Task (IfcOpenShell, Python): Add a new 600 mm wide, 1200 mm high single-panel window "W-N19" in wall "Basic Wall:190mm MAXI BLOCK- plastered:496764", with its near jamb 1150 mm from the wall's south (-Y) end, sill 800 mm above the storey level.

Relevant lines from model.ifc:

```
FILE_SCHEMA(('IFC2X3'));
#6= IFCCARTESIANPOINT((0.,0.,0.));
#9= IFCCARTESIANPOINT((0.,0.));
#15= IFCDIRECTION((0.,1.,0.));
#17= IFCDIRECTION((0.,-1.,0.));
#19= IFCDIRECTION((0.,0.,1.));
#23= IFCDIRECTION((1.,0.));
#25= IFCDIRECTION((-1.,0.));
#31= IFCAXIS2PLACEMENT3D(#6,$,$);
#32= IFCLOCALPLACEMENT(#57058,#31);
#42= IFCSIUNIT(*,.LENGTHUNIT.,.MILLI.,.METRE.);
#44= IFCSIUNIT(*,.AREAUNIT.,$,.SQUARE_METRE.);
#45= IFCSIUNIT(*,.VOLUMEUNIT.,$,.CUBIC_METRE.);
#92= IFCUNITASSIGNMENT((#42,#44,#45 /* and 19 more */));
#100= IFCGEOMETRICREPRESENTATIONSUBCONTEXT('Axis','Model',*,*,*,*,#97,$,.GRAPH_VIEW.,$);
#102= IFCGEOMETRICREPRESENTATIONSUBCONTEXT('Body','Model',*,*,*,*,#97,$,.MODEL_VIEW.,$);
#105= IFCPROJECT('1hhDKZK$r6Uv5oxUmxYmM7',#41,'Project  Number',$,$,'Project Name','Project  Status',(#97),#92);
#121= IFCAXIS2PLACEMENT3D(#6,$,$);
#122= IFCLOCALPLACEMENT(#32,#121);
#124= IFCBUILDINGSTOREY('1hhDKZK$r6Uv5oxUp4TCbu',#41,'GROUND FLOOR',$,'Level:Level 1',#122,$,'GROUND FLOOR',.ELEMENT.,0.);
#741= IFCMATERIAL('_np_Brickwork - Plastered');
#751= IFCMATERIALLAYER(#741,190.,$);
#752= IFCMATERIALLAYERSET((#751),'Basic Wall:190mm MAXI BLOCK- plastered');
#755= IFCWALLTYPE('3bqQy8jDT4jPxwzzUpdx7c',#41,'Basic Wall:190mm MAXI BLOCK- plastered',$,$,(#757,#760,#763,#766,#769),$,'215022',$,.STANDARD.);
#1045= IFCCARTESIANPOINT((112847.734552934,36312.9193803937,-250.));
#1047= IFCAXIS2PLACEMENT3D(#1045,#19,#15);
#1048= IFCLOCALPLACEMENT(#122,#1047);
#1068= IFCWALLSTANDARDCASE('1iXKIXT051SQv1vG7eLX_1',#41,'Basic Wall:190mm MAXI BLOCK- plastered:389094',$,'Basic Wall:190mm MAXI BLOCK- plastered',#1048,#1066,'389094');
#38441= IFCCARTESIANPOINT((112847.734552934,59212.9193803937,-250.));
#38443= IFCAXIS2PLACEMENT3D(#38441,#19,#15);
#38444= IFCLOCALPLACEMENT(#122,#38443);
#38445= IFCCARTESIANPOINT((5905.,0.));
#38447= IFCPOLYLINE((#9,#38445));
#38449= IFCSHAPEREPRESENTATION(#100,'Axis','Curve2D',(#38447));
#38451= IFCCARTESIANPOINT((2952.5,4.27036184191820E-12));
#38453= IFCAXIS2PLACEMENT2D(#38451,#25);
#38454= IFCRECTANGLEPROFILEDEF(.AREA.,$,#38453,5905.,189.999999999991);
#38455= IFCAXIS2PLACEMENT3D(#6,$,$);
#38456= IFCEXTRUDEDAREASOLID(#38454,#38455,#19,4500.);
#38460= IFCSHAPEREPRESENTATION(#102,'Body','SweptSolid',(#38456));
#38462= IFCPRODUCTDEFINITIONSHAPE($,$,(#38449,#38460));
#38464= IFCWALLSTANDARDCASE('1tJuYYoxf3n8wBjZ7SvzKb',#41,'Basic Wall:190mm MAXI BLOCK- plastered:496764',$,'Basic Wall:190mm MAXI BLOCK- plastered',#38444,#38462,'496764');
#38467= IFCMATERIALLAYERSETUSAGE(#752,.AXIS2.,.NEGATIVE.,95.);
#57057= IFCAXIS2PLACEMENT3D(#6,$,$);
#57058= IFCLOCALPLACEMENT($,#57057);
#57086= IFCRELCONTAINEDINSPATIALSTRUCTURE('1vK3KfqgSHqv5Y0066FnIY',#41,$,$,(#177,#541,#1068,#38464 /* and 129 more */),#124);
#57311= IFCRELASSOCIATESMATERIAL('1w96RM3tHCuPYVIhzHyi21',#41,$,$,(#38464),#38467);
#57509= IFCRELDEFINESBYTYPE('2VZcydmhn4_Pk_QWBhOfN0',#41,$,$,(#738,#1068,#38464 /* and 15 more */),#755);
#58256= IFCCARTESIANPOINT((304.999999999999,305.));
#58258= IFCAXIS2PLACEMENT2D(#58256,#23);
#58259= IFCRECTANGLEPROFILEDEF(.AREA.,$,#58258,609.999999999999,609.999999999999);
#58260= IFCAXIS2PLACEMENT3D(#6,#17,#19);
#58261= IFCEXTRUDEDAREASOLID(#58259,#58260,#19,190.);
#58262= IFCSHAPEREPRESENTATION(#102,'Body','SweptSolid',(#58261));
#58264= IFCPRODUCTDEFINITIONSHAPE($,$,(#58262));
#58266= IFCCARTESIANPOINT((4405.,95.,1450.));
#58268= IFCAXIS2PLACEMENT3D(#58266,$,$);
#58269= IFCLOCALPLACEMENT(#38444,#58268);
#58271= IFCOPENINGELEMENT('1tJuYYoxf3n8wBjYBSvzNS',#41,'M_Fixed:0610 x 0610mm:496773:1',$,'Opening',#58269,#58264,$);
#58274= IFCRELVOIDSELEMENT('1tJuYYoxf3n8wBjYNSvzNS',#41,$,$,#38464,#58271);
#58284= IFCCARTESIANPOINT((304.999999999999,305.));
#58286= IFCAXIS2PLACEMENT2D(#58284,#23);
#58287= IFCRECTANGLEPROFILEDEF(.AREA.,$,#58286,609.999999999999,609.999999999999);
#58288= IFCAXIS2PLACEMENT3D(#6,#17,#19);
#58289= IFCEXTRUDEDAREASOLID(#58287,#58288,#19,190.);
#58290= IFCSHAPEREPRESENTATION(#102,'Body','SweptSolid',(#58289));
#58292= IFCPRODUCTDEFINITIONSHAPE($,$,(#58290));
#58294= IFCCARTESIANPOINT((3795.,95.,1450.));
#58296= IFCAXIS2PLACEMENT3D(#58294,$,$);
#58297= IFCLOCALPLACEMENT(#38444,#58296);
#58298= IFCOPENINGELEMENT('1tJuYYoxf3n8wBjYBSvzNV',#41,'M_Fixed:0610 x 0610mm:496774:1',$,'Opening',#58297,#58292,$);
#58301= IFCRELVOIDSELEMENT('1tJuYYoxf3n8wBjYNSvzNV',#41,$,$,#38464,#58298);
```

```python
import numpy as np
import ifcopenshell
import ifcopenshell.api.feature
import ifcopenshell.api.geometry
import ifcopenshell.api.root
import ifcopenshell.api.spatial
import ifcopenshell.api.type
import ifcopenshell.geom
import ifcopenshell.util.element
import ifcopenshell.util.placement
import ifcopenshell.util.representation
import ifcopenshell.util.shape
import ifcopenshell.util.unit

model = ifcopenshell.open("model.ifc")
unit_scale = ifcopenshell.util.unit.calculate_unit_scale(model)
settings = ifcopenshell.geom.settings()


def volume(element):
    """Net volume in cubic metres, openings subtracted."""
    shape = ifcopenshell.geom.create_shape(settings, element)
    return ifcopenshell.util.shape.get_volume(shape.geometry)


wall = model.by_guid("1tJuYYoxf3n8wBjZ7SvzKb")
storey = ifcopenshell.util.element.get_container(wall, ifc_class="IfcBuildingStorey")
context = ifcopenshell.util.representation.get_context(model, "Model", "Body", "MODEL_VIEW")
before = volume(wall)

width, height, from_end, sill = 0.6, 1.2, 1.15, 0.8  # metres

# The wall runs along its own X axis, and the end named is its -X end.
wall_shape = ifcopenshell.geom.create_shape(settings, wall)
x, y, z = ifcopenshell.util.shape.get_vertices(wall_shape.geometry).T
start = x.min() + from_end
face, thickness = float(y.min()), float(y.max() - y.min())
wall_matrix = ifcopenshell.util.placement.get_local_placement(wall.ObjectPlacement)
level = ifcopenshell.util.placement.get_local_placement(storey.ObjectPlacement)[2, 3]


def in_wall(x, y):
    """Placement at x, y metres in the wall's axes, at sill height."""
    matrix = wall_matrix.copy()
    matrix[:, 3] = wall_matrix @ np.array([x / unit_scale, y / unit_scale, 0.0, 1.0])
    matrix[2, 3] = level + sill / unit_scale
    return matrix


# Opening: a box that overshoots both wall faces by 50 mm.
opening = ifcopenshell.api.root.create_entity(model, ifc_class="IfcOpeningElement")
box = ifcopenshell.api.geometry.add_wall_representation(
    model, context=context, length=width, height=height, thickness=thickness + 0.1
)
ifcopenshell.api.geometry.assign_representation(model, product=opening, representation=box)
ifcopenshell.api.geometry.edit_object_placement(model, product=opening, matrix=in_wall(start, face - 0.05), is_si=False)
ifcopenshell.api.feature.add_feature(model, feature=opening, element=wall)

window = ifcopenshell.api.root.create_entity(model, ifc_class="IfcWindow", name="W-N19")
window.OverallWidth, window.OverallHeight = width / unit_scale, height / unit_scale
body = ifcopenshell.api.geometry.add_window_representation(
    model,
    context=context,
    overall_width=window.OverallWidth,
    overall_height=window.OverallHeight,
    partition_type="SINGLE_PANEL",
)
ifcopenshell.api.geometry.assign_representation(model, product=window, representation=body)
ifcopenshell.api.spatial.assign_container(model, products=[window], relating_structure=storey)
fills = ifcopenshell.api.feature.add_filling(model, opening=opening, element=window)
fills.OwnerHistory = window.OwnerHistory  # required in IFC2X3

# IFC2X3 keeps the operation on the window style.
style = ifcopenshell.api.root.create_entity(model, ifc_class="IfcWindowStyle", name="W-N19")
style.OperationType, style.ConstructionType = "SINGLE_PANEL", "NOTDEFINED"
style.ParameterTakesPrecedence = style.Sizeable = False
ifcopenshell.api.type.assign_type(model, related_objects=[window], relating_type=style)

# Centre the window in the wall's thickness.
ifcopenshell.api.geometry.edit_object_placement(model, product=window, matrix=in_wall(start, face), is_si=False)
window_shape = ifcopenshell.geom.create_shape(settings, window)
depth = ifcopenshell.util.shape.get_vertices(window_shape.geometry)[:, 1]
offset = face + thickness / 2 - (depth.min() + depth.max()) / 2
ifcopenshell.api.geometry.edit_object_placement(model, product=window, matrix=in_wall(start, offset), is_si=False)

after = volume(wall)

print(f"wall volume {before:.3f} -> {after:.3f} m3")

model.write("model-out.ifc")
```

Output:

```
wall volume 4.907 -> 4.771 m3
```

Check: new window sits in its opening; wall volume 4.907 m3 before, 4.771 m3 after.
